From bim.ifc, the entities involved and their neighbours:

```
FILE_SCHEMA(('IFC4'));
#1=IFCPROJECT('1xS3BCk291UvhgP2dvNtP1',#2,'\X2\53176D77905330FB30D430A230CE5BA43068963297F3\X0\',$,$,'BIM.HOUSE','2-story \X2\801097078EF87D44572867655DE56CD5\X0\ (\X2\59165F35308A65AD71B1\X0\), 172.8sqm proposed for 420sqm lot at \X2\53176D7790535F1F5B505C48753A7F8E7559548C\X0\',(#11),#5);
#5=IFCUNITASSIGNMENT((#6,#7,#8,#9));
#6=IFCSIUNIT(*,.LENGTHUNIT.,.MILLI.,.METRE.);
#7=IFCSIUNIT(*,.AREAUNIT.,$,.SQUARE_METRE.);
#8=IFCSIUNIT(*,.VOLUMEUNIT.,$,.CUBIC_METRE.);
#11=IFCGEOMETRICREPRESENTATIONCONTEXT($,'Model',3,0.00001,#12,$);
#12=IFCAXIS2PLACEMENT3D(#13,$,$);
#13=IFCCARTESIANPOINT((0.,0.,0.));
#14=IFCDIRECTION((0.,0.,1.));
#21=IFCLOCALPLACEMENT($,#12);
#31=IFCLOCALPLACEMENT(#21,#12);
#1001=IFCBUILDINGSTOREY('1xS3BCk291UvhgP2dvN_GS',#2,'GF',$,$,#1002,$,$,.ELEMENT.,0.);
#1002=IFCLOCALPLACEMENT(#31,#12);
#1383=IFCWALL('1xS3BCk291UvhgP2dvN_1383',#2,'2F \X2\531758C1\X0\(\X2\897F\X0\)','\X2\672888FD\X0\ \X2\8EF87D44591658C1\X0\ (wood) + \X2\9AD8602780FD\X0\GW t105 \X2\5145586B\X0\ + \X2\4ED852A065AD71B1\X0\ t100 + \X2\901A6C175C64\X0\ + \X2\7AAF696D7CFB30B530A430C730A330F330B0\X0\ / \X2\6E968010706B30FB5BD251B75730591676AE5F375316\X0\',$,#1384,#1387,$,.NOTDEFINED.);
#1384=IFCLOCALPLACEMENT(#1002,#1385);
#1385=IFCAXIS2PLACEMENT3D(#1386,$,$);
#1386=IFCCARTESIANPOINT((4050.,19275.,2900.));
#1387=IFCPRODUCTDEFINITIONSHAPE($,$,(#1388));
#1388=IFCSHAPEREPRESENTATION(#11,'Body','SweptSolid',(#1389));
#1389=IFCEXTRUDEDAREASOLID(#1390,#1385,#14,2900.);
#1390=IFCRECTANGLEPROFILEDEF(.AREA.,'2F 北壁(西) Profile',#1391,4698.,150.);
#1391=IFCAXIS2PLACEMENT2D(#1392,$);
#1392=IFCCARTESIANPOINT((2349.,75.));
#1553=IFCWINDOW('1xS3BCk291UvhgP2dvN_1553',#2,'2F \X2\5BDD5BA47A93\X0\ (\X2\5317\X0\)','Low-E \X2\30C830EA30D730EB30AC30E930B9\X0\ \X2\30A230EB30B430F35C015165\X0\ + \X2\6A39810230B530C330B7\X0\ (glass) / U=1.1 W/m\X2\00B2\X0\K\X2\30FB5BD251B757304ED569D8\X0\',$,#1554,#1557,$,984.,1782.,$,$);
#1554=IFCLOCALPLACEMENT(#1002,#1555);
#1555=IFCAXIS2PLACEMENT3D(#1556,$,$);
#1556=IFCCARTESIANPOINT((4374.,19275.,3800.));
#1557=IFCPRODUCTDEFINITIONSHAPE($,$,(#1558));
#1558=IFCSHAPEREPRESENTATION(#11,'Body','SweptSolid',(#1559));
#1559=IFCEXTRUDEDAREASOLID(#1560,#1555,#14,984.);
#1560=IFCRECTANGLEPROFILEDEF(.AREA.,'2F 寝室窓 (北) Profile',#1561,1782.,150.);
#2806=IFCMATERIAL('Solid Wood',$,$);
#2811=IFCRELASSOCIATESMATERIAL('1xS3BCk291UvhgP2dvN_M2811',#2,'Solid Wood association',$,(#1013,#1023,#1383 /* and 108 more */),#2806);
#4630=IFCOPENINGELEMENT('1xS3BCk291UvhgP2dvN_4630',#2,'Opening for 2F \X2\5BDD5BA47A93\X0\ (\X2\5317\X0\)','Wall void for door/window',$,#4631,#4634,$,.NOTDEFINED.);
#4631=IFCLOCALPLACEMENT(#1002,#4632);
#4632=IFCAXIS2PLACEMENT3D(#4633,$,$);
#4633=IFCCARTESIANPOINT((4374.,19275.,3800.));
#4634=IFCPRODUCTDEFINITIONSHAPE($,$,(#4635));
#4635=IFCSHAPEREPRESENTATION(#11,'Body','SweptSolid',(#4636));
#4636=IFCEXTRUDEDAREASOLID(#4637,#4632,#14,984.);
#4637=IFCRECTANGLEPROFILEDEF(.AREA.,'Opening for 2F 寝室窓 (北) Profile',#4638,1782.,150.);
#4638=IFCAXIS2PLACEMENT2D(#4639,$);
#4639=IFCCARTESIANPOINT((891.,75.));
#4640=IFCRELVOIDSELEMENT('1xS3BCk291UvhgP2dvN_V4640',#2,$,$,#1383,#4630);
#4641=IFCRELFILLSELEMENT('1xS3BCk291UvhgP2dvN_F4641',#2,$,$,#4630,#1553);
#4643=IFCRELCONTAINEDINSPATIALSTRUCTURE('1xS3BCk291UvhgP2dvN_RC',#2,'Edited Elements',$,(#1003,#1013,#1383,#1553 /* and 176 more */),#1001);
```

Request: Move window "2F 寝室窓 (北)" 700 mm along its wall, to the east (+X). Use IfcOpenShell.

```python
import ifcopenshell
import ifcopenshell.api.geometry
import ifcopenshell.util.placement
import ifcopenshell.util.unit

model = ifcopenshell.open("bim.ifc")
unit_scale = ifcopenshell.util.unit.calculate_unit_scale(model)

window = model.by_guid("1xS3BCk291UvhgP2dvN_1553")
opening = window.FillsVoids[0].RelatingOpeningElement
wall = opening.VoidsElements[0].RelatingBuildingElement

wall_matrix = ifcopenshell.util.placement.get_local_placement(wall.ObjectPlacement)
shift = wall_matrix[:3, 0] * 0.7 / unit_scale
before = ifcopenshell.util.placement.get_local_placement(window.ObjectPlacement)[:3, 3].copy()

# The window is not placed relative to its opening, so move both.
for product in (opening, window):
    matrix = ifcopenshell.util.placement.get_local_placement(product.ObjectPlacement)
    matrix[:3, 3] += shift
    ifcopenshell.api.geometry.edit_object_placement(model, product=product, matrix=matrix, is_si=False)

after = ifcopenshell.util.placement.get_local_placement(window.ObjectPlacement)[:3, 3]
print("window moved by", (after - before).round(3) + 0.0)

model.write("bim_updated.ifc")
```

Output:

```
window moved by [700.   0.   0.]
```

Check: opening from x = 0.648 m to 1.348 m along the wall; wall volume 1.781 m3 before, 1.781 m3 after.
